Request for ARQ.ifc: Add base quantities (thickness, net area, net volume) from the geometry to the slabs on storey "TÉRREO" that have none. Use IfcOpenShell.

First a look at what the model holds.

```python
import ifcopenshell
import ifcopenshell.util.element
import ifcopenshell.util.unit

model = ifcopenshell.open("ARQ.ifc")
print(model.schema)
for unit_type in ("LENGTHUNIT", "AREAUNIT", "VOLUMEUNIT"):
    print(unit_type, ifcopenshell.util.unit.calculate_unit_scale(model, unit_type))
storey = next(s for s in model.by_type("IfcBuildingStorey") if s.Name == "TÉRREO")
slabs = [e for e in ifcopenshell.util.element.get_decomposition(storey) if e.is_a("IfcSlab")]
for e in sorted(slabs, key=lambda e: e.id()):
    print(e.id(), e.is_a(), e.Name, list(ifcopenshell.util.element.get_psets(e, qtos_only=True)), sep=" | ")
```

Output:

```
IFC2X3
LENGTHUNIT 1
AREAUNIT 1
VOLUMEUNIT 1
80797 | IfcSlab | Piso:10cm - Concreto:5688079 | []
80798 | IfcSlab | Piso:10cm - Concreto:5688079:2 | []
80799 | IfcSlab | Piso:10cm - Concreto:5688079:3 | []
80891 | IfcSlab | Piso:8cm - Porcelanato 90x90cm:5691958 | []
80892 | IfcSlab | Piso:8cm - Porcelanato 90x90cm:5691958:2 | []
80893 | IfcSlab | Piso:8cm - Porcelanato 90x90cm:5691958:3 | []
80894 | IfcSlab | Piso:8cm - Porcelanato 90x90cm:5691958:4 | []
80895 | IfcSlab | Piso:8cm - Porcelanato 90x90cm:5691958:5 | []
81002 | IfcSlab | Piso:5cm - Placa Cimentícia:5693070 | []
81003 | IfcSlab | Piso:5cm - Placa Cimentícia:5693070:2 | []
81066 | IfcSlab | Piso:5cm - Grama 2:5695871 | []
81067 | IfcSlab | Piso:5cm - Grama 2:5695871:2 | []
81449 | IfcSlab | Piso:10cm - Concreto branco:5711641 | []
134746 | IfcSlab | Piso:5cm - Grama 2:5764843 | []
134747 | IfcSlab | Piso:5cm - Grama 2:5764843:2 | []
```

```python
import ifcopenshell
import ifcopenshell.api.pset
import ifcopenshell.geom
import ifcopenshell.util.element
import ifcopenshell.util.shape
import ifcopenshell.util.unit

model = ifcopenshell.open("ARQ.ifc")
unit_scale = ifcopenshell.util.unit.calculate_unit_scale(model)
area_scale = ifcopenshell.util.unit.calculate_unit_scale(model, "AREAUNIT")
volume_scale = ifcopenshell.util.unit.calculate_unit_scale(model, "VOLUMEUNIT")
settings = ifcopenshell.geom.settings()

storey = next(s for s in model.by_type("IfcBuildingStorey") if s.Name == "TÉRREO")
slabs = [e for e in ifcopenshell.util.element.get_decomposition(storey) if e.is_a("IfcSlab")]

for e in sorted(slabs, key=lambda e: e.id()):
    if ifcopenshell.util.element.get_psets(e, qtos_only=True, should_inherit=False):
        continue
    # Geometry comes back in metres, in the element's own axes.
    shape = ifcopenshell.geom.create_shape(settings, e)
    values = {
        "Width": ifcopenshell.util.shape.get_z(shape.geometry) / unit_scale,
        "NetArea": ifcopenshell.util.shape.get_footprint_area(shape.geometry) / area_scale,
        "NetVolume": ifcopenshell.util.shape.get_volume(shape.geometry) / volume_scale,
    }
    qto = ifcopenshell.api.pset.add_qto(model, product=e, name="BaseQuantities")
    ifcopenshell.api.pset.edit_qto(model, qto=qto, properties=values)
    print(e.id(), {k: round(v, 3) for k, v in values.items()})

model.write("ARQ_v2.ifc")
```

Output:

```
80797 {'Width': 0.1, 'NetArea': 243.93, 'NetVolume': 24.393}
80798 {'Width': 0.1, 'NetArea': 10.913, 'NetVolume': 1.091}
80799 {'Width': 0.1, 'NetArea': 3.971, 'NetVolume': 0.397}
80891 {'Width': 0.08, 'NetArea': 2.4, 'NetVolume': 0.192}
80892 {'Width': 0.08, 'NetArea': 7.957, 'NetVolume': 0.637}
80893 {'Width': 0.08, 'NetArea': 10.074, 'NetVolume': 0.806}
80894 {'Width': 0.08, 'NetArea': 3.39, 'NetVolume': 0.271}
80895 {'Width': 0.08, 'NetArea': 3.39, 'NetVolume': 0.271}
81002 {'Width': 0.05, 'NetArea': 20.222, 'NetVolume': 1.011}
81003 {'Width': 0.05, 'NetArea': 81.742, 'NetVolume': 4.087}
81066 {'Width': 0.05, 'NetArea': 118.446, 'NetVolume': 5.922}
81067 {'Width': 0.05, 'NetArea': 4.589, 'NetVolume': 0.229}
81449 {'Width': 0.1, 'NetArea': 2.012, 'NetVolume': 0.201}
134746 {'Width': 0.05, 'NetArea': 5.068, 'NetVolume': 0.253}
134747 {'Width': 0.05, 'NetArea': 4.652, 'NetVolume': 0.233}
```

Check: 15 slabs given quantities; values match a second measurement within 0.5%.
